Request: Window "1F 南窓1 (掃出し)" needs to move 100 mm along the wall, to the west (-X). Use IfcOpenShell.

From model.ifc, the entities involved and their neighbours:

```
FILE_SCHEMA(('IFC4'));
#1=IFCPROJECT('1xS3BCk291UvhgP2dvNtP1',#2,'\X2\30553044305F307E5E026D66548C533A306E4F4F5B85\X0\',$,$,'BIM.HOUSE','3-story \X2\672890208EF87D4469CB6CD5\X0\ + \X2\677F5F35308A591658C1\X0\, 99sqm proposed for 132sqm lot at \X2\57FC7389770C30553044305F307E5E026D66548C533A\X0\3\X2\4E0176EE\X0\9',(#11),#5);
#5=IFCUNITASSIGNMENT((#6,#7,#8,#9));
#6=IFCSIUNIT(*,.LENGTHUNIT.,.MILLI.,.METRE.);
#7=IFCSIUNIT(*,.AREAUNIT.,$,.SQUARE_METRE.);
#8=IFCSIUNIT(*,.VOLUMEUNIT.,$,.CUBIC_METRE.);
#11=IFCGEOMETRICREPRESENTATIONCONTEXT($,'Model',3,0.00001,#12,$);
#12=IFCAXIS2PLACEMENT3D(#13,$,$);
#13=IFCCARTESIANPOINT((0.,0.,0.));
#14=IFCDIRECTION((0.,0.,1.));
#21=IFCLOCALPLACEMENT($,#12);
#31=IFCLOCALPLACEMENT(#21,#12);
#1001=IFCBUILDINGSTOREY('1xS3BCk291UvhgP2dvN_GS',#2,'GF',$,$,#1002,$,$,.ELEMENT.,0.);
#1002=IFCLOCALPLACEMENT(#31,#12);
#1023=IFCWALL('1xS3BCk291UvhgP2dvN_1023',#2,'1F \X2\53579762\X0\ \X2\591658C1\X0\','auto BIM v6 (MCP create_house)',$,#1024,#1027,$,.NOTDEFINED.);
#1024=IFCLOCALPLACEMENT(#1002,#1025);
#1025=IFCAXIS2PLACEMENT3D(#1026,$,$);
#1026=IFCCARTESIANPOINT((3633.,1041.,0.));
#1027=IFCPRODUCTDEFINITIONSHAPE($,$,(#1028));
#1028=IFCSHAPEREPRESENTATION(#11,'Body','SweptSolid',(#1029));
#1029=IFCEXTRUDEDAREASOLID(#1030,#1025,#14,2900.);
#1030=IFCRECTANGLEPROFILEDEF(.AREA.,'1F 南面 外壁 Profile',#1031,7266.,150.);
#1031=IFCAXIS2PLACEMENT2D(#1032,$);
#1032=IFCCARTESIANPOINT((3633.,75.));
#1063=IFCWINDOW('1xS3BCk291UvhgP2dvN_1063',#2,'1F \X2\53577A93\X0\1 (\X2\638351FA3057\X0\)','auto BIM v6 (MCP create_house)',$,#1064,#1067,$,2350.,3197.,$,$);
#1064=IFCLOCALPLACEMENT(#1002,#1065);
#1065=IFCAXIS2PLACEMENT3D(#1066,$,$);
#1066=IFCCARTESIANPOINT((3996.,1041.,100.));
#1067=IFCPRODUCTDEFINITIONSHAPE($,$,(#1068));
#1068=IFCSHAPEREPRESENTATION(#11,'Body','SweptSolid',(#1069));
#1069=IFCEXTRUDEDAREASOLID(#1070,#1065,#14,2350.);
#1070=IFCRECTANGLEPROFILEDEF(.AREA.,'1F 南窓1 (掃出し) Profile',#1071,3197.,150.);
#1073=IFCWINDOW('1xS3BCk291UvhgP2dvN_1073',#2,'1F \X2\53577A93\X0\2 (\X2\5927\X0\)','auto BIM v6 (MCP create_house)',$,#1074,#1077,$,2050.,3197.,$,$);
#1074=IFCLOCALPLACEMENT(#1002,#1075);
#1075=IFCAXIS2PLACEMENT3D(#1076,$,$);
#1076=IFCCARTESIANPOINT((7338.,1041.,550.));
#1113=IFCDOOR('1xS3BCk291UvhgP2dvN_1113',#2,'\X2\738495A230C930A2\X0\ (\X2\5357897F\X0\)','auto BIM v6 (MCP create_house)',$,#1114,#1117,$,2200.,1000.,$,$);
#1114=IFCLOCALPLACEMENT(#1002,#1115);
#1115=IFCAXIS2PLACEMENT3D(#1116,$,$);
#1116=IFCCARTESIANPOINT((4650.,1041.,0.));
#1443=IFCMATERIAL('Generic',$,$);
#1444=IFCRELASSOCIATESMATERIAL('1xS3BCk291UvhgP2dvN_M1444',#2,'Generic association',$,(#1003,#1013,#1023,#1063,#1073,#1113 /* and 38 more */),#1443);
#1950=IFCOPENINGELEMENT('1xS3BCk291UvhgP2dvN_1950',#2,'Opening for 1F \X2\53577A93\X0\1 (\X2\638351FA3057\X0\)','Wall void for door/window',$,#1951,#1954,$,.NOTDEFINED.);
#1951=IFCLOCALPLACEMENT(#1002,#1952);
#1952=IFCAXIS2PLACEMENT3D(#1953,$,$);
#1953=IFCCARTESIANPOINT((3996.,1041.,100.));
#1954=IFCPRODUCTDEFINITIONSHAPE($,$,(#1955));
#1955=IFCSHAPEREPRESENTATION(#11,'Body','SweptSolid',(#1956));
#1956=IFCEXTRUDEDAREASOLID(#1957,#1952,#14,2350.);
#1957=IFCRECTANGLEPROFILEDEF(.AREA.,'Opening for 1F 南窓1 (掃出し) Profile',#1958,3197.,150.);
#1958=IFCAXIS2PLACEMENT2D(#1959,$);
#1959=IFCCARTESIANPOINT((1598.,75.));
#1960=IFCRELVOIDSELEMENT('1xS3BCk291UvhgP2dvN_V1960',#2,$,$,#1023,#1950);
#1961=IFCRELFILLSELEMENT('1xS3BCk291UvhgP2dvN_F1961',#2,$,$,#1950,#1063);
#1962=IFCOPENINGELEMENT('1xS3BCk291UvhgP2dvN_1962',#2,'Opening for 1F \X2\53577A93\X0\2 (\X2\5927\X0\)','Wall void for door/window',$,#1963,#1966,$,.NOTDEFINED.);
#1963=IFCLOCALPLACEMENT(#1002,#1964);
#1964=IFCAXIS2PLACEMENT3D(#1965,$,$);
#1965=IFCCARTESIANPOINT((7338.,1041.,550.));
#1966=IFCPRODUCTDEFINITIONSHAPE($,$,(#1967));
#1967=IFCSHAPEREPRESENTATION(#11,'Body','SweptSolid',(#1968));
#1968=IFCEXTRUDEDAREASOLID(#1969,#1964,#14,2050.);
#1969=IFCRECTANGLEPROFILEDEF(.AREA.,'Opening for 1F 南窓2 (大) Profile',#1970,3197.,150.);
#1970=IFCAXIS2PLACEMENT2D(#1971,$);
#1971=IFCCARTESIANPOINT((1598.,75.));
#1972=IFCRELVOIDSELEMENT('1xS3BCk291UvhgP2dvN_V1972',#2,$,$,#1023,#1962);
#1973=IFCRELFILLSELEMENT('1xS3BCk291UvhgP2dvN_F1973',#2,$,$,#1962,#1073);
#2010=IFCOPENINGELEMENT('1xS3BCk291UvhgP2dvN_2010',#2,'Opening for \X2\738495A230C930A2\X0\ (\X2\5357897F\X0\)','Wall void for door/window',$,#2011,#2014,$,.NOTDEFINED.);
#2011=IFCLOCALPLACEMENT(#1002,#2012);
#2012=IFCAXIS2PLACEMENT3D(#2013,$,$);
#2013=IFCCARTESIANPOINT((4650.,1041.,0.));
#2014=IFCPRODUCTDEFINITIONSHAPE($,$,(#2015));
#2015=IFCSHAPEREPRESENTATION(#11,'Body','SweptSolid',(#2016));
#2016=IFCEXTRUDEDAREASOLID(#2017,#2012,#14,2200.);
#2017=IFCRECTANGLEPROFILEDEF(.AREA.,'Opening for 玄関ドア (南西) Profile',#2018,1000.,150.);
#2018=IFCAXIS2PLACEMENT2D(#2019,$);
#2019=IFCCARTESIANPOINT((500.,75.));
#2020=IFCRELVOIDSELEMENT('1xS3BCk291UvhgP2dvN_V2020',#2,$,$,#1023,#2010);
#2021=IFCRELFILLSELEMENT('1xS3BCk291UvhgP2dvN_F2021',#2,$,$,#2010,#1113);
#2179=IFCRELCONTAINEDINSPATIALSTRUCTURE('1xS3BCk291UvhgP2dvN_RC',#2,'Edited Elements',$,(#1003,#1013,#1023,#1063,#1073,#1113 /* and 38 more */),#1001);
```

```python
import ifcopenshell
import ifcopenshell.api.geometry
import ifcopenshell.util.placement
import ifcopenshell.util.unit

model = ifcopenshell.open("model.ifc")
unit_scale = ifcopenshell.util.unit.calculate_unit_scale(model)

window = model.by_id(1063)
opening = window.FillsVoids[0].RelatingOpeningElement
wall = opening.VoidsElements[0].RelatingBuildingElement

wall_matrix = ifcopenshell.util.placement.get_local_placement(wall.ObjectPlacement)
shift = wall_matrix[:3, 0] * -0.1 / unit_scale
before = ifcopenshell.util.placement.get_local_placement(window.ObjectPlacement)[:3, 3].copy()

# The window is not placed relative to its opening, so move both.
for product in (opening, window):
    matrix = ifcopenshell.util.placement.get_local_placement(product.ObjectPlacement)
    matrix[:3, 3] += shift
    ifcopenshell.api.geometry.edit_object_placement(model, product=product, matrix=matrix, is_si=False)

after = ifcopenshell.util.placement.get_local_placement(window.ObjectPlacement)[:3, 3]
print("window moved by", (after - before).round(3) + 0.0)

model.write("model-out.ifc")
```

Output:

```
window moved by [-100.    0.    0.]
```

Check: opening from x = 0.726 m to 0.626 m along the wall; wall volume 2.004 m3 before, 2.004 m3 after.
